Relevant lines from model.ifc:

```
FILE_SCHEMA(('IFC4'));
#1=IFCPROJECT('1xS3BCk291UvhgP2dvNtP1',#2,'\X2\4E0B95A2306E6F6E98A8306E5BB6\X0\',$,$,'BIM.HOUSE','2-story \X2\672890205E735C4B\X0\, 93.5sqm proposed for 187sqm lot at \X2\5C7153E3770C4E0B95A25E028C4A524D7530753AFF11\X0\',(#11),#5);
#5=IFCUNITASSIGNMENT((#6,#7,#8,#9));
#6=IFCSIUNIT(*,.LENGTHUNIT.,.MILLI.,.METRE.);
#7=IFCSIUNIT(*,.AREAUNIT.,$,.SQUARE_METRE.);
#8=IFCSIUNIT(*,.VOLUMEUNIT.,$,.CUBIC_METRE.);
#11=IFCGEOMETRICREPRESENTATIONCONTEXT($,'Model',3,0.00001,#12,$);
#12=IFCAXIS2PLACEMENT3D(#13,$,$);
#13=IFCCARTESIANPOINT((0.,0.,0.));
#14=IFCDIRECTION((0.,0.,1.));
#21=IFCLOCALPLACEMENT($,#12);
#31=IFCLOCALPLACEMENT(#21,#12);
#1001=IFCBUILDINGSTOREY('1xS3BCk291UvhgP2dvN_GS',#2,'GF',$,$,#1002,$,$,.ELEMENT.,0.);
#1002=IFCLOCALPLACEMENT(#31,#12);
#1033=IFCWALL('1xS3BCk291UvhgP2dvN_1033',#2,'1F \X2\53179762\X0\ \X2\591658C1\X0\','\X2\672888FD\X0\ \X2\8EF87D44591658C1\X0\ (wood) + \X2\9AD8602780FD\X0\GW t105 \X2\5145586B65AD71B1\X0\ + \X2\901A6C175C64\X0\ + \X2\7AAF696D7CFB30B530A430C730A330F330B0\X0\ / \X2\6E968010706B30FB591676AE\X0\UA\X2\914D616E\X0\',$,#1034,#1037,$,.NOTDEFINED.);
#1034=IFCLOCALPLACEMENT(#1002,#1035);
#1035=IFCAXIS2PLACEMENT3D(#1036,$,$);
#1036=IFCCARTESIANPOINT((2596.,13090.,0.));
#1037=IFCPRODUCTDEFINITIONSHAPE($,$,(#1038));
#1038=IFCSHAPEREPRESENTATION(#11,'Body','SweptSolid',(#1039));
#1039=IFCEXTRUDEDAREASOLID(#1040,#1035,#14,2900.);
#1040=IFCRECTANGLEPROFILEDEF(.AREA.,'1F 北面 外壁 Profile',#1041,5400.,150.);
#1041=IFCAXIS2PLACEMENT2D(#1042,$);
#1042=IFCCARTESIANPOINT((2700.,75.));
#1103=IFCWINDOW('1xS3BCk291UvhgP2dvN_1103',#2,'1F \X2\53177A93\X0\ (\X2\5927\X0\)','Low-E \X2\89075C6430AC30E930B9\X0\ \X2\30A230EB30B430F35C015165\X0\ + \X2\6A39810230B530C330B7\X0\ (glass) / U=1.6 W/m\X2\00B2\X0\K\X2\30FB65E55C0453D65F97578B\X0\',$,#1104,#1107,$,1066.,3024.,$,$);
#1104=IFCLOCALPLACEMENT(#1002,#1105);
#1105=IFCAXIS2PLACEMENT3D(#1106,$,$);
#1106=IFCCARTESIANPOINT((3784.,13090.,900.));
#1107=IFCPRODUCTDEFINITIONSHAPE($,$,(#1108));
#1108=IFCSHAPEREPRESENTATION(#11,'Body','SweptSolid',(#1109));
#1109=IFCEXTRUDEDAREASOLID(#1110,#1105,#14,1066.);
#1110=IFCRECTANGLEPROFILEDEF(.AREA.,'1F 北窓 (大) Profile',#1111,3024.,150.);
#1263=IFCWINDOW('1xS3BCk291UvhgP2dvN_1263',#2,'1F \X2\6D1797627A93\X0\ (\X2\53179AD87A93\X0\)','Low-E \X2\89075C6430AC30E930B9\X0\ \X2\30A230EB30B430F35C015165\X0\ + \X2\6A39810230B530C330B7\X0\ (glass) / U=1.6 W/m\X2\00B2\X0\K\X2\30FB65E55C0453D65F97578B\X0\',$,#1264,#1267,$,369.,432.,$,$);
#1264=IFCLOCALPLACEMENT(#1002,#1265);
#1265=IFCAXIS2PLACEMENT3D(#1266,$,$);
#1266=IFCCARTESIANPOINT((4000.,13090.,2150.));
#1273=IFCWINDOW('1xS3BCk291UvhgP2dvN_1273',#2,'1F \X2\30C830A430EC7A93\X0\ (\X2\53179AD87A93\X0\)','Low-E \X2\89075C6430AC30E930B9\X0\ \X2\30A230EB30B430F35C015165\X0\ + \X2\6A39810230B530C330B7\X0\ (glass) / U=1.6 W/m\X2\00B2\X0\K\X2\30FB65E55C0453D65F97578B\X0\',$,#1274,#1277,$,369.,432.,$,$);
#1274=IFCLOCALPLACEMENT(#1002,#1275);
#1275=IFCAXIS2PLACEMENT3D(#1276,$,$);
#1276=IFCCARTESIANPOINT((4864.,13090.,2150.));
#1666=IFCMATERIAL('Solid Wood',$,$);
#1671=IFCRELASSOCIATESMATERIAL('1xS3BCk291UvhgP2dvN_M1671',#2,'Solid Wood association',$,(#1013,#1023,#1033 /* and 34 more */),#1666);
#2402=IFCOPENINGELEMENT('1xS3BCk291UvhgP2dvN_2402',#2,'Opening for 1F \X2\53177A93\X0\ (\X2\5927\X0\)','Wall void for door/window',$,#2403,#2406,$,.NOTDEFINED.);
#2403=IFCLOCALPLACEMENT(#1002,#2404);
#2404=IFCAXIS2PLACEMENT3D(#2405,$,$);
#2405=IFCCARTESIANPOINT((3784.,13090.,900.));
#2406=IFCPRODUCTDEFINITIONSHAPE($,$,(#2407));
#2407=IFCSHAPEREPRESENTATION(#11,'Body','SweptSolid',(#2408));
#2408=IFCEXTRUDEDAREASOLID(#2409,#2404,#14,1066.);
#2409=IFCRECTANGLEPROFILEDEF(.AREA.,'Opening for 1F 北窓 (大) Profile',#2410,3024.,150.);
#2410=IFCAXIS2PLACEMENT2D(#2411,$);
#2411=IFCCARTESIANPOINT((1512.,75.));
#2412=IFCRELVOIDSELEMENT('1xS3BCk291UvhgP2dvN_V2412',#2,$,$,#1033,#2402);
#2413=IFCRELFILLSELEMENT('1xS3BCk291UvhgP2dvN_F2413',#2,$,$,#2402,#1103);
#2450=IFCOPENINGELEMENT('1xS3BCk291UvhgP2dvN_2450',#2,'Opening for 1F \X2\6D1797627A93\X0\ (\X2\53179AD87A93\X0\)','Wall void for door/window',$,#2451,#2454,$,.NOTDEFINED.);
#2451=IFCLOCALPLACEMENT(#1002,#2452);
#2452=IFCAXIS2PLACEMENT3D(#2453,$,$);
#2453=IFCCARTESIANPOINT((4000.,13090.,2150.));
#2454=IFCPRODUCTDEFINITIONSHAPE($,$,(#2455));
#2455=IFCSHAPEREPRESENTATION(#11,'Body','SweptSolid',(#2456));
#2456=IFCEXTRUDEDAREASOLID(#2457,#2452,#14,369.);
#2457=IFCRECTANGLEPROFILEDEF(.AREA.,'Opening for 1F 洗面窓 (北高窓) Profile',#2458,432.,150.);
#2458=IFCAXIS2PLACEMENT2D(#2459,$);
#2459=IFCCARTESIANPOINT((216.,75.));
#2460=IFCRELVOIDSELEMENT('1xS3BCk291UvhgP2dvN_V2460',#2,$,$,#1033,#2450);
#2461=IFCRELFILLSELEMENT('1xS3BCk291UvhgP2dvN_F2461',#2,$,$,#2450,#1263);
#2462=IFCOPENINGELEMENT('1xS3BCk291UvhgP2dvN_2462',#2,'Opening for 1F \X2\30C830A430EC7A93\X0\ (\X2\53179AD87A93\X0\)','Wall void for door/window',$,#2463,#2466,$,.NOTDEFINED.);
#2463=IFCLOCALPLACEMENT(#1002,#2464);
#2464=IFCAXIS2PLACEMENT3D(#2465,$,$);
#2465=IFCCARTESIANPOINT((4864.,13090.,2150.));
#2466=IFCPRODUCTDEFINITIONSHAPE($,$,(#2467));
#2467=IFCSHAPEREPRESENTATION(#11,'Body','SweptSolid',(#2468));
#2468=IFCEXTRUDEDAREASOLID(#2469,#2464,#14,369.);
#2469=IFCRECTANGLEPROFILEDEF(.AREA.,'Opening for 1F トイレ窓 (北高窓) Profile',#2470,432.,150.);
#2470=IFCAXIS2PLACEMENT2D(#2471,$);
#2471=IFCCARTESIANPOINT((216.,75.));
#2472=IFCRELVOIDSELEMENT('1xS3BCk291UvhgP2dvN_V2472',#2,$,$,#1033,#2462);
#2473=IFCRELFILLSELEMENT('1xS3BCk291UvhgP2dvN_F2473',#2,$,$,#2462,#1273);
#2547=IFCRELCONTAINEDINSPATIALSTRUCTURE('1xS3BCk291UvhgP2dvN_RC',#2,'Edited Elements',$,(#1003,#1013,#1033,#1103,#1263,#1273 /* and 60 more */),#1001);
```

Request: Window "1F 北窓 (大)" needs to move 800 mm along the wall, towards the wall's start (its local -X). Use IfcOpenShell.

```python
import ifcopenshell
import ifcopenshell.api.geometry
import ifcopenshell.util.placement

model = ifcopenshell.open("model.ifc")

window = model.by_guid("1xS3BCk291UvhgP2dvN_1103")
opening = window.FillsVoids[0].RelatingOpeningElement
wall = opening.VoidsElements[0].RelatingBuildingElement

wall_matrix = ifcopenshell.util.placement.get_local_placement(wall.ObjectPlacement)
shift = wall_matrix[:3, 0] * -800.0
before = ifcopenshell.util.placement.get_local_placement(window.ObjectPlacement)[:3, 3].copy()

# The window is not placed relative to its opening, so move both.
for product in (opening, window):
    matrix = ifcopenshell.util.placement.get_local_placement(product.ObjectPlacement)
    matrix[:3, 3] += shift
    ifcopenshell.api.geometry.edit_object_placement(model, product=product, matrix=matrix, is_si=False)

after = ifcopenshell.util.placement.get_local_placement(window.ObjectPlacement)[:3, 3]
print("window moved by", (after - before).round(3) + 0.0)

model.write("model_v2.ifc")
```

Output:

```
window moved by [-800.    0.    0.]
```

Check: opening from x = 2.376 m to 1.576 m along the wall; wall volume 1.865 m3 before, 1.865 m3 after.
